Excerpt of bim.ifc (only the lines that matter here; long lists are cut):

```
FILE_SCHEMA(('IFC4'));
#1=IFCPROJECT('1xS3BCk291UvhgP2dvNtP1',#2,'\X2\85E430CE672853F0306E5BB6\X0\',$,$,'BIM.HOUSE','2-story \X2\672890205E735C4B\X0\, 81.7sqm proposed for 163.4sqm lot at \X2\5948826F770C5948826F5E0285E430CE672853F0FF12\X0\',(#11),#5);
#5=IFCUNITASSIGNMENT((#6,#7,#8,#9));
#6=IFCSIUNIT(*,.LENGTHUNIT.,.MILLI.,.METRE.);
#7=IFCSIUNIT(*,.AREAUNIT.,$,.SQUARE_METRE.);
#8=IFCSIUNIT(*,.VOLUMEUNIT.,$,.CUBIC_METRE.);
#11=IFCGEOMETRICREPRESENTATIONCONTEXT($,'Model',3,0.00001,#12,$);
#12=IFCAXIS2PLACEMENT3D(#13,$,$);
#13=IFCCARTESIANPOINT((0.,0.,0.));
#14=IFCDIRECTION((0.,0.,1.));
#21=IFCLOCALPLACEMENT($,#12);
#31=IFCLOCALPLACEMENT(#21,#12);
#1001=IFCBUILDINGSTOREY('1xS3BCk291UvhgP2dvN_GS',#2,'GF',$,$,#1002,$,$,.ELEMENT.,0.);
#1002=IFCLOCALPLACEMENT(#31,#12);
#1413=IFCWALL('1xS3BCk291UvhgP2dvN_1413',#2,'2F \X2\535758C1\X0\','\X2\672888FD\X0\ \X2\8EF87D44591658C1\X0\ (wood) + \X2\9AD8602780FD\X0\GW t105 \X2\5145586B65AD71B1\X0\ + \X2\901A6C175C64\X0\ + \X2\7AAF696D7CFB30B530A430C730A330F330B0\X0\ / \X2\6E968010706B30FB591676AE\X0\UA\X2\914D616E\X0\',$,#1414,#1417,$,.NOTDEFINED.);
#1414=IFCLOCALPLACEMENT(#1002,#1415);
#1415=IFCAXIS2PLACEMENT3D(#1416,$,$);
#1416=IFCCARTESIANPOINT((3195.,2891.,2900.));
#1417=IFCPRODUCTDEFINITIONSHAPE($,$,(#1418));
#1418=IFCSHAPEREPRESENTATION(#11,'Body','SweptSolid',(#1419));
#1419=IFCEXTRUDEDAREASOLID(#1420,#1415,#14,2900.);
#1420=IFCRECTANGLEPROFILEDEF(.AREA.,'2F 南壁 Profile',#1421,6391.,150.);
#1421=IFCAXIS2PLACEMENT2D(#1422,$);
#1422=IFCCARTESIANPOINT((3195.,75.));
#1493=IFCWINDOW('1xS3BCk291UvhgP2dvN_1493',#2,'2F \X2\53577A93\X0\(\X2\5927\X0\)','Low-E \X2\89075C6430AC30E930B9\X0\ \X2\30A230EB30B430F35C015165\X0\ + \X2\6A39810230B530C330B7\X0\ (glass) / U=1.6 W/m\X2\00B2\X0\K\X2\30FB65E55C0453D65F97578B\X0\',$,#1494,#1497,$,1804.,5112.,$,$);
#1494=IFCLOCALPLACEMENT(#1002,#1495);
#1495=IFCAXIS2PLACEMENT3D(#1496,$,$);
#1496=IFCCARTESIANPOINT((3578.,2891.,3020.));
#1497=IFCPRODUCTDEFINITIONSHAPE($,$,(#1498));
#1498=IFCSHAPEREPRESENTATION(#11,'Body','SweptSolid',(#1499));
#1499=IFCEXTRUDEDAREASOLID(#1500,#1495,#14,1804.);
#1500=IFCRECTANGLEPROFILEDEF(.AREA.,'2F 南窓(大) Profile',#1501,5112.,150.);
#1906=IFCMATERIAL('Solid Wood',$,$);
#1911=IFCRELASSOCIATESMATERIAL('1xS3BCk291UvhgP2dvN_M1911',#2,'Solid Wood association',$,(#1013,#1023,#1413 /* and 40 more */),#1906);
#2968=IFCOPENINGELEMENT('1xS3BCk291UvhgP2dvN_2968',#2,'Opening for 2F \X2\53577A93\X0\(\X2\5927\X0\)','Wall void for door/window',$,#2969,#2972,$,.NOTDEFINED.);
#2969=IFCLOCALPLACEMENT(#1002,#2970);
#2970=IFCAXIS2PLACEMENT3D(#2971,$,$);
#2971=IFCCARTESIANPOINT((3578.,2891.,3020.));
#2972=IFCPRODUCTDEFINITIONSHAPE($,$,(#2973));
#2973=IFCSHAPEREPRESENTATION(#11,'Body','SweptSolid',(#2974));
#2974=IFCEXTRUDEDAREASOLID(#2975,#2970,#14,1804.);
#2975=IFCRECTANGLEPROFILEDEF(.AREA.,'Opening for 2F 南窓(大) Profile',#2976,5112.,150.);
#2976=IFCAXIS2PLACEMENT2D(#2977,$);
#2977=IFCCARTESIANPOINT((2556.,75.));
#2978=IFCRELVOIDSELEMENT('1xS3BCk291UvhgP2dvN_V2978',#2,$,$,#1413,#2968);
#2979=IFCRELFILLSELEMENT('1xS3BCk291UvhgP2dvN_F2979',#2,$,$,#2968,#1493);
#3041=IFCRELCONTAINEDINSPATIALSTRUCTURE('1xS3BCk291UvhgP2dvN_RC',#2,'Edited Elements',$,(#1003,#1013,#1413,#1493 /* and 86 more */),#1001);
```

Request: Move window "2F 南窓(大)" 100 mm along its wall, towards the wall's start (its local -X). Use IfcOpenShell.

```python
import ifcopenshell
import ifcopenshell.api.geometry
import ifcopenshell.util.placement
import ifcopenshell.util.unit

model = ifcopenshell.open("bim.ifc")
unit_scale = ifcopenshell.util.unit.calculate_unit_scale(model)

window = model.by_id(1493)
opening = window.FillsVoids[0].RelatingOpeningElement
wall = opening.VoidsElements[0].RelatingBuildingElement

wall_matrix = ifcopenshell.util.placement.get_local_placement(wall.ObjectPlacement)
shift = wall_matrix[:3, 0] * -0.1 / unit_scale
before = ifcopenshell.util.placement.get_local_placement(window.ObjectPlacement)[:3, 3].copy()

# The window is not placed relative to its opening, so move both.
for product in (opening, window):
    matrix = ifcopenshell.util.placement.get_local_placement(product.ObjectPlacement)
    matrix[:3, 3] += shift
    ifcopenshell.api.geometry.edit_object_placement(model, product=product, matrix=matrix, is_si=False)

after = ifcopenshell.util.placement.get_local_placement(window.ObjectPlacement)[:3, 3]
print("window moved by", (after - before).round(3) + 0.0)

model.write("bim_edited.ifc")
```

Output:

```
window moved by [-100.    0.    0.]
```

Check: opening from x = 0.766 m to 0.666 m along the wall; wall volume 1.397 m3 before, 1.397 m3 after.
